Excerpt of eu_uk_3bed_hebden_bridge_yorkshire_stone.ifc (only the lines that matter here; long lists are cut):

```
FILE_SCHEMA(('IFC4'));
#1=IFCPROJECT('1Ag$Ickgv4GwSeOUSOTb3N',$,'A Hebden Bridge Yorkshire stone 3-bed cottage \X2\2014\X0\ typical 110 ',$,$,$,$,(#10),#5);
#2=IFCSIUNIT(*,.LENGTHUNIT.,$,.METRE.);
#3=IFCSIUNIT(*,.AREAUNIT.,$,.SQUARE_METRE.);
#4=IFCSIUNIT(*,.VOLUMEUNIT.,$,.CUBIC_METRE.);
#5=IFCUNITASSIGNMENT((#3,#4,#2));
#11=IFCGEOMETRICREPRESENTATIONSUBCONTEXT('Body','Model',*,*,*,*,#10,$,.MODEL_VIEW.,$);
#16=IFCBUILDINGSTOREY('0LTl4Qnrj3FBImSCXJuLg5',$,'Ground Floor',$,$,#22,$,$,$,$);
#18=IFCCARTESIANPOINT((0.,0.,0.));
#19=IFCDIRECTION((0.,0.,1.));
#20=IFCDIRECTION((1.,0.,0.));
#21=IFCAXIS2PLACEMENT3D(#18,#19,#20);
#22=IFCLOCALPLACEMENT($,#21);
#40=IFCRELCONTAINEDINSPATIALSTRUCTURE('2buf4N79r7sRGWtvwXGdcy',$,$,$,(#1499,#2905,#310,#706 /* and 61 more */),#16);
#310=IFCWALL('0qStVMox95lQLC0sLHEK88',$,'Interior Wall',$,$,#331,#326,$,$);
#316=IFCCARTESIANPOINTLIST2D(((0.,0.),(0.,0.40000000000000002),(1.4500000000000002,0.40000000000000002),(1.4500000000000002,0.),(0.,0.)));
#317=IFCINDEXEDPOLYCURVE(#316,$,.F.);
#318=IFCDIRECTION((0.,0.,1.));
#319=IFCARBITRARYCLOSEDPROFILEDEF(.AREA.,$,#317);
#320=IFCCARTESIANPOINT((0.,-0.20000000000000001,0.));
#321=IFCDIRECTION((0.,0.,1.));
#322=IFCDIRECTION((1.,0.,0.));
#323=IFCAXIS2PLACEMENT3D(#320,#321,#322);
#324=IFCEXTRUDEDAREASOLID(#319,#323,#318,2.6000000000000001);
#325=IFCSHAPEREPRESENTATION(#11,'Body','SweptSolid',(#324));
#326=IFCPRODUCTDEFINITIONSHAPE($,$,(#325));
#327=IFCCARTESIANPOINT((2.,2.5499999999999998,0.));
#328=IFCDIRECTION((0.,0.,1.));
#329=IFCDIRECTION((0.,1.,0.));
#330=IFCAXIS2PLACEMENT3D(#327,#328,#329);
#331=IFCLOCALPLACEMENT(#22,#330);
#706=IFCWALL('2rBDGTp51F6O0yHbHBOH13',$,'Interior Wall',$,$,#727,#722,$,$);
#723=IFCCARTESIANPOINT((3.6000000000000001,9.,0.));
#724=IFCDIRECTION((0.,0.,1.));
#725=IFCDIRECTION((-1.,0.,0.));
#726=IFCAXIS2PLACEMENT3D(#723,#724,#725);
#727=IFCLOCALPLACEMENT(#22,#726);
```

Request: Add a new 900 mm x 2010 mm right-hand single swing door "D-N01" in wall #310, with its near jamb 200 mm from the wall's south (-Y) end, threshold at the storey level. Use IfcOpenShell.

```python
import numpy as np
import ifcopenshell
import ifcopenshell.api.feature
import ifcopenshell.api.geometry
import ifcopenshell.api.root
import ifcopenshell.api.spatial
import ifcopenshell.geom
import ifcopenshell.util.element
import ifcopenshell.util.placement
import ifcopenshell.util.representation
import ifcopenshell.util.shape
import ifcopenshell.util.unit

model = ifcopenshell.open("eu_uk_3bed_hebden_bridge_yorkshire_stone.ifc")
unit_scale = ifcopenshell.util.unit.calculate_unit_scale(model)
settings = ifcopenshell.geom.settings()


def volume(element):
    """Net volume in cubic metres, openings subtracted."""
    shape = ifcopenshell.geom.create_shape(settings, element)
    return ifcopenshell.util.shape.get_volume(shape.geometry)


wall = model.by_id(310)
storey = ifcopenshell.util.element.get_container(wall, ifc_class="IfcBuildingStorey")
context = ifcopenshell.util.representation.get_context(model, "Model", "Body", "MODEL_VIEW")
before = volume(wall)

width, height, from_end, sill = 0.9, 2.01, 0.2, 0.0  # metres

# The wall runs along its own X axis, and the end named is its -X end.
wall_shape = ifcopenshell.geom.create_shape(settings, wall)
x, y, z = ifcopenshell.util.shape.get_vertices(wall_shape.geometry).T
start = x.min() + from_end
face, thickness = float(y.min()), float(y.max() - y.min())
wall_matrix = ifcopenshell.util.placement.get_local_placement(wall.ObjectPlacement)
level = ifcopenshell.util.placement.get_local_placement(storey.ObjectPlacement)[2, 3]


def in_wall(x, y):
    """Placement at x, y metres in the wall's axes, at sill height."""
    matrix = wall_matrix.copy()
    matrix[:, 3] = wall_matrix @ np.array([x / unit_scale, y / unit_scale, 0.0, 1.0])
    matrix[2, 3] = level + sill / unit_scale
    return matrix


# Opening: a box that overshoots both wall faces by 50 mm.
opening = ifcopenshell.api.root.create_entity(model, ifc_class="IfcOpeningElement", predefined_type="OPENING")
box = ifcopenshell.api.geometry.add_wall_representation(
    model, context=context, length=width, height=height, thickness=thickness + 0.1
)
ifcopenshell.api.geometry.assign_representation(model, product=opening, representation=box)
ifcopenshell.api.geometry.edit_object_placement(model, product=opening, matrix=in_wall(start, face - 0.05), is_si=False)
ifcopenshell.api.feature.add_feature(model, feature=opening, element=wall)

door = ifcopenshell.api.root.create_entity(model, ifc_class="IfcDoor", name="D-N01", predefined_type="DOOR")
door.OverallWidth, door.OverallHeight = width / unit_scale, height / unit_scale
door.OperationType = "SINGLE_SWING_RIGHT"
body = ifcopenshell.api.geometry.add_door_representation(
    model,
    context=context,
    overall_width=door.OverallWidth,
    overall_height=door.OverallHeight,
    operation_type="SINGLE_SWING_RIGHT",
    lining_properties={"LiningDepth": thickness / unit_scale, "ThresholdDepth": thickness / unit_scale},
)
ifcopenshell.api.geometry.assign_representation(model, product=door, representation=body)
ifcopenshell.api.spatial.assign_container(model, products=[door], relating_structure=storey)
ifcopenshell.api.feature.add_filling(model, opening=opening, element=door)

# The lining spans the wall, so the door starts at the wall face.
ifcopenshell.api.geometry.edit_object_placement(model, product=door, matrix=in_wall(start, face), is_si=False)

after = volume(wall)

print(f"wall volume {before:.3f} -> {after:.3f} m3")

model.write("eu_uk_3bed_hebden_bridge_yorkshire_stone_updated.ifc")
```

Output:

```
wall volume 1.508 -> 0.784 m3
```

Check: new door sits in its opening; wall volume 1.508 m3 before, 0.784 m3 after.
